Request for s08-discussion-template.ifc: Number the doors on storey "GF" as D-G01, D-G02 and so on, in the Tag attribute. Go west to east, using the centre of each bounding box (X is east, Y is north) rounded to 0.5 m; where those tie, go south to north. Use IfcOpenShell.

First a look at what the model holds.

```python
import ifcopenshell
import ifcopenshell.util.element
import ifcopenshell.util.placement

model = ifcopenshell.open("s08-discussion-template.ifc")
print(model.schema)
storey = next(s for s in model.by_type("IfcBuildingStorey") if s.Name == "GF")
doors = [e for e in ifcopenshell.util.element.get_decomposition(storey) if e.is_a("IfcDoor")]
for e in sorted(doors, key=lambda e: e.id()):
    origin = ifcopenshell.util.placement.get_local_placement(e.ObjectPlacement)[:3, 3]
    print(e.id(), e.Tag, e.Name, origin.round(2) + 0.0, sep=" | ")
```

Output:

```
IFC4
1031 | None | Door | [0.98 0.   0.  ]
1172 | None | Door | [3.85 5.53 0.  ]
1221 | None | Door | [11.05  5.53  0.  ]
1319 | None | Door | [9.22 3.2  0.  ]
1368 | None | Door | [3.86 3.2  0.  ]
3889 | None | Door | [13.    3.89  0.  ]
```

```python
import ifcopenshell
import ifcopenshell.geom
import ifcopenshell.util.element
import ifcopenshell.util.shape

model = ifcopenshell.open("s08-discussion-template.ifc")
settings = ifcopenshell.geom.settings()
settings.set("use-world-coords", True)


def centre(element):
    shape = ifcopenshell.geom.create_shape(settings, element)
    return ifcopenshell.util.shape.get_bbox_centroid(shape.geometry)


storey = next(s for s in model.by_type("IfcBuildingStorey") if s.Name == "GF")
doors = [e for e in ifcopenshell.util.element.get_decomposition(storey) if e.is_a("IfcDoor")]

# Insertion points can sit at a corner or the storey origin, so sort by the geometry (in metres).
centres = {e: centre(e) for e in doors}
doors.sort(key=lambda e: (round(centres[e][0] / 0.5), centres[e][1]))

for i, e in enumerate(doors, start=1):
    number = f"D-G{i:02d}"
    e.Tag = number
    print(e.id(), number)

model.write("s08-discussion-template-out.ifc")
```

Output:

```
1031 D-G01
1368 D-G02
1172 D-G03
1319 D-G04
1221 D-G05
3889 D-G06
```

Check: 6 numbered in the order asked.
